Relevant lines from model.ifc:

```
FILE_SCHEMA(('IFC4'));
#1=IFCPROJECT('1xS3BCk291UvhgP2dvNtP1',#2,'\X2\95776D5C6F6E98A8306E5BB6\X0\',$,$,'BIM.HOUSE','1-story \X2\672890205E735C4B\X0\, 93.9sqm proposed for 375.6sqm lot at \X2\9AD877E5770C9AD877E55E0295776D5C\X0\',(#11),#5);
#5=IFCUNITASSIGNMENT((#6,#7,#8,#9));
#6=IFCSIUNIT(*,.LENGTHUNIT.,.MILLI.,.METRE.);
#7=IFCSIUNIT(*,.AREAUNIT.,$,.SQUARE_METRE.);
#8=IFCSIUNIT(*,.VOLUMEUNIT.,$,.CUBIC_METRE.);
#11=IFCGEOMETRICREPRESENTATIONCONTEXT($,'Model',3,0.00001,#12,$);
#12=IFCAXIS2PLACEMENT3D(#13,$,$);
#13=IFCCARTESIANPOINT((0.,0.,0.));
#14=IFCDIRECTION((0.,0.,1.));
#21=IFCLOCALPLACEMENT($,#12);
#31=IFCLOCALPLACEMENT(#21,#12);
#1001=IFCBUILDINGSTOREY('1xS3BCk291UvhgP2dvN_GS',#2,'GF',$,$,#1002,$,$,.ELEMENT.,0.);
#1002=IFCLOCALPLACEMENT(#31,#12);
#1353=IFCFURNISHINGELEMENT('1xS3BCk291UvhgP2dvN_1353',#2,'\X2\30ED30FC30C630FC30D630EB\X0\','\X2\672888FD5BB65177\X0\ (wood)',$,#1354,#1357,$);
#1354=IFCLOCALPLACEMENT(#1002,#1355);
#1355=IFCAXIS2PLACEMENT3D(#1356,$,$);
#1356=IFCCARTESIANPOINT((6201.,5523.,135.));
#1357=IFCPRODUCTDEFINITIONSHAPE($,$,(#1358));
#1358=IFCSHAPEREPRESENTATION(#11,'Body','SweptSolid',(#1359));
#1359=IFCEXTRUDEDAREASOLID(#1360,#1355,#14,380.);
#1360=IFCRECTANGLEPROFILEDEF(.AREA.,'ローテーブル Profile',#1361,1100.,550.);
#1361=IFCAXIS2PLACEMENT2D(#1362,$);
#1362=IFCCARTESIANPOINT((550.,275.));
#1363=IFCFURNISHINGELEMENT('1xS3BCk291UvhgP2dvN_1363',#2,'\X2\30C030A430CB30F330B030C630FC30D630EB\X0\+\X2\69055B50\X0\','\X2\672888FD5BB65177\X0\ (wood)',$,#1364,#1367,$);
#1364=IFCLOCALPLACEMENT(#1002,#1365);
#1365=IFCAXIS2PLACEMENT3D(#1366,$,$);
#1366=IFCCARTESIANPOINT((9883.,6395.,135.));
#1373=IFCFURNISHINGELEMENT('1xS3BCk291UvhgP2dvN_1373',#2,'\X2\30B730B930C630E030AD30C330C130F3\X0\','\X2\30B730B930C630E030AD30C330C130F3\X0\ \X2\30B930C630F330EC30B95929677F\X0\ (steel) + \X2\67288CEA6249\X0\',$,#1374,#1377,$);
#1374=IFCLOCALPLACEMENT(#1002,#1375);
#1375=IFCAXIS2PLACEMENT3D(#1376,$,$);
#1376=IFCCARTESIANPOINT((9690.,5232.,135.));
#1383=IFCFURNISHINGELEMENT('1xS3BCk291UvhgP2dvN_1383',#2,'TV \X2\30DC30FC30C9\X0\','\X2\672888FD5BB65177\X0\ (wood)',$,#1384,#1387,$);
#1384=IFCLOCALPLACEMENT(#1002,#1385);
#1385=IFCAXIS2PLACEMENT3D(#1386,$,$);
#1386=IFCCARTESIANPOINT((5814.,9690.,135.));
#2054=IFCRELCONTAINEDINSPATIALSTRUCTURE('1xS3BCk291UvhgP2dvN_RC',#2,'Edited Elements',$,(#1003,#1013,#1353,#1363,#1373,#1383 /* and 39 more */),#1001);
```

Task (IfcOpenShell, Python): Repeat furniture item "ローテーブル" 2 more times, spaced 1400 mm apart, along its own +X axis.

```python
import ifcopenshell
import ifcopenshell.api.geometry
import ifcopenshell.api.root
import ifcopenshell.util.element
import ifcopenshell.util.placement
import ifcopenshell.util.unit

model = ifcopenshell.open("model.ifc")
unit_scale = ifcopenshell.util.unit.calculate_unit_scale(model)


def reuse_history(source, copy):
    """copy_class also copies each property set's owner history, people and application; keep the originals."""
    for rel in copy.IsDefinedBy:
        if rel.is_a("IfcRelDefinesByProperties") and (history := rel.RelatingPropertyDefinition.OwnerHistory):
            rel.RelatingPropertyDefinition.OwnerHistory = source.OwnerHistory
            ifcopenshell.util.element.remove_deep2(model, history)


source = model.by_id(1353)
base = ifcopenshell.util.placement.get_local_placement(source.ObjectPlacement)
step = base[:3, 0] * 1.4 / unit_scale

for i in range(1, 3):
    copy = ifcopenshell.api.root.copy_class(model, product=source)
    copy.Representation = ifcopenshell.util.element.copy_deep(
        model, source.Representation, exclude=["IfcGeometricRepresentationContext", "IfcRepresentationMap"]
    )
    reuse_history(source, copy)
    matrix = base.copy()
    matrix[:3, 3] += i * step
    print("added at", matrix[:3, 3].round(3) + 0.0)
    ifcopenshell.api.geometry.edit_object_placement(model, product=copy, matrix=matrix, is_si=False)

model.write("model_v2.ifc")
```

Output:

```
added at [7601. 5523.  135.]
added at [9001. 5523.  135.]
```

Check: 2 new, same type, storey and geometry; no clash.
